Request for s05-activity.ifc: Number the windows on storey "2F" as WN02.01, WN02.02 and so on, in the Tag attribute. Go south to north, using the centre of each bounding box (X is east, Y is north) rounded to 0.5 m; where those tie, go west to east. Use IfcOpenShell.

First a look at what the model holds.

```python
import ifcopenshell
import ifcopenshell.util.element
import ifcopenshell.util.placement

model = ifcopenshell.open("s05-activity.ifc")
print(model.schema)
storey = next(s for s in model.by_type("IfcBuildingStorey") if s.Name == "2F")
windows = [e for e in ifcopenshell.util.element.get_decomposition(storey) if e.is_a("IfcWindow")]
for e in sorted(windows, key=lambda e: e.id()):
    origin = ifcopenshell.util.placement.get_local_placement(e.ObjectPlacement)[:3, 3]
    print(e.id(), e.Tag, e.Name, origin.round(2) + 0.0, sep=" | ")
```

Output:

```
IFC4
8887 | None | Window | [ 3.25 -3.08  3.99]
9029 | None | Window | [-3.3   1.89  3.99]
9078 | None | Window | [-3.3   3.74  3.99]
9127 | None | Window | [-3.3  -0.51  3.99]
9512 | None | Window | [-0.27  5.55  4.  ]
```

```python
import ifcopenshell
import ifcopenshell.geom
import ifcopenshell.util.element
import ifcopenshell.util.shape

model = ifcopenshell.open("s05-activity.ifc")
settings = ifcopenshell.geom.settings()
settings.set("use-world-coords", True)


def centre(element):
    shape = ifcopenshell.geom.create_shape(settings, element)
    return ifcopenshell.util.shape.get_bbox_centroid(shape.geometry)


storey = next(s for s in model.by_type("IfcBuildingStorey") if s.Name == "2F")
windows = [e for e in ifcopenshell.util.element.get_decomposition(storey) if e.is_a("IfcWindow")]

# Insertion points can sit at a corner or the storey origin, so sort by the geometry (in metres).
centres = {e: centre(e) for e in windows}
windows.sort(key=lambda e: (round(centres[e][1] / 0.5), centres[e][0]))

for i, e in enumerate(windows, start=1):
    number = f"WN02.{i:02d}"
    e.Tag = number
    print(e.id(), number)

model.write("s05-activity_rev.ifc")
```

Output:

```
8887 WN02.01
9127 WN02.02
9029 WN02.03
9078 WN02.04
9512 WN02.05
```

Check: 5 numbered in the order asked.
